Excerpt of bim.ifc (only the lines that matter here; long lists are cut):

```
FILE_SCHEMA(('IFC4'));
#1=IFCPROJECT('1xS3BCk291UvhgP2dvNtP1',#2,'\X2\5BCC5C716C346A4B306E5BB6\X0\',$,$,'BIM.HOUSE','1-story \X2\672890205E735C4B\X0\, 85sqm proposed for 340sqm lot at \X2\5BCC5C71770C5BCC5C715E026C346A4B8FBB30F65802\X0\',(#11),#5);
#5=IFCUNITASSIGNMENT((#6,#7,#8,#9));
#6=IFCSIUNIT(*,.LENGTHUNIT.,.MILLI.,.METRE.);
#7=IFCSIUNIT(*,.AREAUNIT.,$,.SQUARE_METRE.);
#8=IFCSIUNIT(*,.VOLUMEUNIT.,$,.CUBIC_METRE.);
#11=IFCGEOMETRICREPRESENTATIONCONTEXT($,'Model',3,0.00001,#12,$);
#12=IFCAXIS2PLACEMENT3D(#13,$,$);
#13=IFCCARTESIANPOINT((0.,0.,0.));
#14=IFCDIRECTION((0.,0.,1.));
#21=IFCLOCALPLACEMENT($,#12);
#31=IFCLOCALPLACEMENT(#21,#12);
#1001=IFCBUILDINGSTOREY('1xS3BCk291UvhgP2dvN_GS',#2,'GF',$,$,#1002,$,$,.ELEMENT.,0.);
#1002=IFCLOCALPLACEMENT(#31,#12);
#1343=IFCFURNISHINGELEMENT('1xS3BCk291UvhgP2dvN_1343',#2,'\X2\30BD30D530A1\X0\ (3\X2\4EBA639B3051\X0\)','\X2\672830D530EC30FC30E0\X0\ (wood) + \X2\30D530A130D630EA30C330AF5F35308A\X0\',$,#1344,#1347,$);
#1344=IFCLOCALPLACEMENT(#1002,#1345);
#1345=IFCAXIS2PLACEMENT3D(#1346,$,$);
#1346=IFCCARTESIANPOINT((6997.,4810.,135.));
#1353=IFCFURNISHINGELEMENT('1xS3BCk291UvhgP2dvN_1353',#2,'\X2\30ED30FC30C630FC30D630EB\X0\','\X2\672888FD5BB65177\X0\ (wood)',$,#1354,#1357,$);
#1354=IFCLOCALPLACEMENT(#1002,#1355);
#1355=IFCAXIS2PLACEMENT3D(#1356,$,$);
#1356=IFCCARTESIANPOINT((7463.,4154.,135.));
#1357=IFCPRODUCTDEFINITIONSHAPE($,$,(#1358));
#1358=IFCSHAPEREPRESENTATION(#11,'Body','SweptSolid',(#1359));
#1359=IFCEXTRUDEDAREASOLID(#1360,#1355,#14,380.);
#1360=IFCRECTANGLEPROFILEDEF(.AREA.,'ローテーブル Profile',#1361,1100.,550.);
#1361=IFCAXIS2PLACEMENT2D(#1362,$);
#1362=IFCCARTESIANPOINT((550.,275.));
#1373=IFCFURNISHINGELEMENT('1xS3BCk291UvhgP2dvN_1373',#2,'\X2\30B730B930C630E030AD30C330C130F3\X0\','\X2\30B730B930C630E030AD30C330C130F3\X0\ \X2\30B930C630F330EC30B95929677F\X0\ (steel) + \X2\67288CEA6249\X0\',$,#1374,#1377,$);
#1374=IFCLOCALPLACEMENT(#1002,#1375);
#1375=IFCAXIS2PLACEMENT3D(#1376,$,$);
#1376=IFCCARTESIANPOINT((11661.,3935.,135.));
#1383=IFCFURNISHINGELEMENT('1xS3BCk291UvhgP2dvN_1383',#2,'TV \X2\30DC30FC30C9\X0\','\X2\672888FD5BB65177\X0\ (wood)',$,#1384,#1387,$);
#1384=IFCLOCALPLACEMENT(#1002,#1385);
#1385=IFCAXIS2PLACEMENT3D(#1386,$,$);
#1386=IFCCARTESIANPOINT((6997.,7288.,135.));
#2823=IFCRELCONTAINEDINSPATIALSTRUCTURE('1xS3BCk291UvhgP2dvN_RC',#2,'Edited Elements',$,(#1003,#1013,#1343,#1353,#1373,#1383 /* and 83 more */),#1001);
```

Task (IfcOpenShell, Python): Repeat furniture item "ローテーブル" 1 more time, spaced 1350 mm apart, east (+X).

```python
import numpy as np
import ifcopenshell
import ifcopenshell.api.geometry
import ifcopenshell.api.root
import ifcopenshell.util.element
import ifcopenshell.util.placement
import ifcopenshell.util.unit

model = ifcopenshell.open("bim.ifc")
unit_scale = ifcopenshell.util.unit.calculate_unit_scale(model)


def reuse_history(source, copy):
    """copy_class also copies each property set's owner history, people and application; keep the originals."""
    for rel in copy.IsDefinedBy:
        if rel.is_a("IfcRelDefinesByProperties") and (history := rel.RelatingPropertyDefinition.OwnerHistory):
            rel.RelatingPropertyDefinition.OwnerHistory = source.OwnerHistory
            ifcopenshell.util.element.remove_deep2(model, history)


source = model.by_guid("1xS3BCk291UvhgP2dvN_1353")
base = ifcopenshell.util.placement.get_local_placement(source.ObjectPlacement)
step = np.array([1.0, 0.0, 0.0]) * 1.35 / unit_scale

for i in range(1, 2):
    copy = ifcopenshell.api.root.copy_class(model, product=source)
    copy.Representation = ifcopenshell.util.element.copy_deep(
        model, source.Representation, exclude=["IfcGeometricRepresentationContext", "IfcRepresentationMap"]
    )
    reuse_history(source, copy)
    matrix = base.copy()
    matrix[:3, 3] += i * step
    print("added at", matrix[:3, 3].round(3) + 0.0)
    ifcopenshell.api.geometry.edit_object_placement(model, product=copy, matrix=matrix, is_si=False)

model.write("bim_rev.ifc")
```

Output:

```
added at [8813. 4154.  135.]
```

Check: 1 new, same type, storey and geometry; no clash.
